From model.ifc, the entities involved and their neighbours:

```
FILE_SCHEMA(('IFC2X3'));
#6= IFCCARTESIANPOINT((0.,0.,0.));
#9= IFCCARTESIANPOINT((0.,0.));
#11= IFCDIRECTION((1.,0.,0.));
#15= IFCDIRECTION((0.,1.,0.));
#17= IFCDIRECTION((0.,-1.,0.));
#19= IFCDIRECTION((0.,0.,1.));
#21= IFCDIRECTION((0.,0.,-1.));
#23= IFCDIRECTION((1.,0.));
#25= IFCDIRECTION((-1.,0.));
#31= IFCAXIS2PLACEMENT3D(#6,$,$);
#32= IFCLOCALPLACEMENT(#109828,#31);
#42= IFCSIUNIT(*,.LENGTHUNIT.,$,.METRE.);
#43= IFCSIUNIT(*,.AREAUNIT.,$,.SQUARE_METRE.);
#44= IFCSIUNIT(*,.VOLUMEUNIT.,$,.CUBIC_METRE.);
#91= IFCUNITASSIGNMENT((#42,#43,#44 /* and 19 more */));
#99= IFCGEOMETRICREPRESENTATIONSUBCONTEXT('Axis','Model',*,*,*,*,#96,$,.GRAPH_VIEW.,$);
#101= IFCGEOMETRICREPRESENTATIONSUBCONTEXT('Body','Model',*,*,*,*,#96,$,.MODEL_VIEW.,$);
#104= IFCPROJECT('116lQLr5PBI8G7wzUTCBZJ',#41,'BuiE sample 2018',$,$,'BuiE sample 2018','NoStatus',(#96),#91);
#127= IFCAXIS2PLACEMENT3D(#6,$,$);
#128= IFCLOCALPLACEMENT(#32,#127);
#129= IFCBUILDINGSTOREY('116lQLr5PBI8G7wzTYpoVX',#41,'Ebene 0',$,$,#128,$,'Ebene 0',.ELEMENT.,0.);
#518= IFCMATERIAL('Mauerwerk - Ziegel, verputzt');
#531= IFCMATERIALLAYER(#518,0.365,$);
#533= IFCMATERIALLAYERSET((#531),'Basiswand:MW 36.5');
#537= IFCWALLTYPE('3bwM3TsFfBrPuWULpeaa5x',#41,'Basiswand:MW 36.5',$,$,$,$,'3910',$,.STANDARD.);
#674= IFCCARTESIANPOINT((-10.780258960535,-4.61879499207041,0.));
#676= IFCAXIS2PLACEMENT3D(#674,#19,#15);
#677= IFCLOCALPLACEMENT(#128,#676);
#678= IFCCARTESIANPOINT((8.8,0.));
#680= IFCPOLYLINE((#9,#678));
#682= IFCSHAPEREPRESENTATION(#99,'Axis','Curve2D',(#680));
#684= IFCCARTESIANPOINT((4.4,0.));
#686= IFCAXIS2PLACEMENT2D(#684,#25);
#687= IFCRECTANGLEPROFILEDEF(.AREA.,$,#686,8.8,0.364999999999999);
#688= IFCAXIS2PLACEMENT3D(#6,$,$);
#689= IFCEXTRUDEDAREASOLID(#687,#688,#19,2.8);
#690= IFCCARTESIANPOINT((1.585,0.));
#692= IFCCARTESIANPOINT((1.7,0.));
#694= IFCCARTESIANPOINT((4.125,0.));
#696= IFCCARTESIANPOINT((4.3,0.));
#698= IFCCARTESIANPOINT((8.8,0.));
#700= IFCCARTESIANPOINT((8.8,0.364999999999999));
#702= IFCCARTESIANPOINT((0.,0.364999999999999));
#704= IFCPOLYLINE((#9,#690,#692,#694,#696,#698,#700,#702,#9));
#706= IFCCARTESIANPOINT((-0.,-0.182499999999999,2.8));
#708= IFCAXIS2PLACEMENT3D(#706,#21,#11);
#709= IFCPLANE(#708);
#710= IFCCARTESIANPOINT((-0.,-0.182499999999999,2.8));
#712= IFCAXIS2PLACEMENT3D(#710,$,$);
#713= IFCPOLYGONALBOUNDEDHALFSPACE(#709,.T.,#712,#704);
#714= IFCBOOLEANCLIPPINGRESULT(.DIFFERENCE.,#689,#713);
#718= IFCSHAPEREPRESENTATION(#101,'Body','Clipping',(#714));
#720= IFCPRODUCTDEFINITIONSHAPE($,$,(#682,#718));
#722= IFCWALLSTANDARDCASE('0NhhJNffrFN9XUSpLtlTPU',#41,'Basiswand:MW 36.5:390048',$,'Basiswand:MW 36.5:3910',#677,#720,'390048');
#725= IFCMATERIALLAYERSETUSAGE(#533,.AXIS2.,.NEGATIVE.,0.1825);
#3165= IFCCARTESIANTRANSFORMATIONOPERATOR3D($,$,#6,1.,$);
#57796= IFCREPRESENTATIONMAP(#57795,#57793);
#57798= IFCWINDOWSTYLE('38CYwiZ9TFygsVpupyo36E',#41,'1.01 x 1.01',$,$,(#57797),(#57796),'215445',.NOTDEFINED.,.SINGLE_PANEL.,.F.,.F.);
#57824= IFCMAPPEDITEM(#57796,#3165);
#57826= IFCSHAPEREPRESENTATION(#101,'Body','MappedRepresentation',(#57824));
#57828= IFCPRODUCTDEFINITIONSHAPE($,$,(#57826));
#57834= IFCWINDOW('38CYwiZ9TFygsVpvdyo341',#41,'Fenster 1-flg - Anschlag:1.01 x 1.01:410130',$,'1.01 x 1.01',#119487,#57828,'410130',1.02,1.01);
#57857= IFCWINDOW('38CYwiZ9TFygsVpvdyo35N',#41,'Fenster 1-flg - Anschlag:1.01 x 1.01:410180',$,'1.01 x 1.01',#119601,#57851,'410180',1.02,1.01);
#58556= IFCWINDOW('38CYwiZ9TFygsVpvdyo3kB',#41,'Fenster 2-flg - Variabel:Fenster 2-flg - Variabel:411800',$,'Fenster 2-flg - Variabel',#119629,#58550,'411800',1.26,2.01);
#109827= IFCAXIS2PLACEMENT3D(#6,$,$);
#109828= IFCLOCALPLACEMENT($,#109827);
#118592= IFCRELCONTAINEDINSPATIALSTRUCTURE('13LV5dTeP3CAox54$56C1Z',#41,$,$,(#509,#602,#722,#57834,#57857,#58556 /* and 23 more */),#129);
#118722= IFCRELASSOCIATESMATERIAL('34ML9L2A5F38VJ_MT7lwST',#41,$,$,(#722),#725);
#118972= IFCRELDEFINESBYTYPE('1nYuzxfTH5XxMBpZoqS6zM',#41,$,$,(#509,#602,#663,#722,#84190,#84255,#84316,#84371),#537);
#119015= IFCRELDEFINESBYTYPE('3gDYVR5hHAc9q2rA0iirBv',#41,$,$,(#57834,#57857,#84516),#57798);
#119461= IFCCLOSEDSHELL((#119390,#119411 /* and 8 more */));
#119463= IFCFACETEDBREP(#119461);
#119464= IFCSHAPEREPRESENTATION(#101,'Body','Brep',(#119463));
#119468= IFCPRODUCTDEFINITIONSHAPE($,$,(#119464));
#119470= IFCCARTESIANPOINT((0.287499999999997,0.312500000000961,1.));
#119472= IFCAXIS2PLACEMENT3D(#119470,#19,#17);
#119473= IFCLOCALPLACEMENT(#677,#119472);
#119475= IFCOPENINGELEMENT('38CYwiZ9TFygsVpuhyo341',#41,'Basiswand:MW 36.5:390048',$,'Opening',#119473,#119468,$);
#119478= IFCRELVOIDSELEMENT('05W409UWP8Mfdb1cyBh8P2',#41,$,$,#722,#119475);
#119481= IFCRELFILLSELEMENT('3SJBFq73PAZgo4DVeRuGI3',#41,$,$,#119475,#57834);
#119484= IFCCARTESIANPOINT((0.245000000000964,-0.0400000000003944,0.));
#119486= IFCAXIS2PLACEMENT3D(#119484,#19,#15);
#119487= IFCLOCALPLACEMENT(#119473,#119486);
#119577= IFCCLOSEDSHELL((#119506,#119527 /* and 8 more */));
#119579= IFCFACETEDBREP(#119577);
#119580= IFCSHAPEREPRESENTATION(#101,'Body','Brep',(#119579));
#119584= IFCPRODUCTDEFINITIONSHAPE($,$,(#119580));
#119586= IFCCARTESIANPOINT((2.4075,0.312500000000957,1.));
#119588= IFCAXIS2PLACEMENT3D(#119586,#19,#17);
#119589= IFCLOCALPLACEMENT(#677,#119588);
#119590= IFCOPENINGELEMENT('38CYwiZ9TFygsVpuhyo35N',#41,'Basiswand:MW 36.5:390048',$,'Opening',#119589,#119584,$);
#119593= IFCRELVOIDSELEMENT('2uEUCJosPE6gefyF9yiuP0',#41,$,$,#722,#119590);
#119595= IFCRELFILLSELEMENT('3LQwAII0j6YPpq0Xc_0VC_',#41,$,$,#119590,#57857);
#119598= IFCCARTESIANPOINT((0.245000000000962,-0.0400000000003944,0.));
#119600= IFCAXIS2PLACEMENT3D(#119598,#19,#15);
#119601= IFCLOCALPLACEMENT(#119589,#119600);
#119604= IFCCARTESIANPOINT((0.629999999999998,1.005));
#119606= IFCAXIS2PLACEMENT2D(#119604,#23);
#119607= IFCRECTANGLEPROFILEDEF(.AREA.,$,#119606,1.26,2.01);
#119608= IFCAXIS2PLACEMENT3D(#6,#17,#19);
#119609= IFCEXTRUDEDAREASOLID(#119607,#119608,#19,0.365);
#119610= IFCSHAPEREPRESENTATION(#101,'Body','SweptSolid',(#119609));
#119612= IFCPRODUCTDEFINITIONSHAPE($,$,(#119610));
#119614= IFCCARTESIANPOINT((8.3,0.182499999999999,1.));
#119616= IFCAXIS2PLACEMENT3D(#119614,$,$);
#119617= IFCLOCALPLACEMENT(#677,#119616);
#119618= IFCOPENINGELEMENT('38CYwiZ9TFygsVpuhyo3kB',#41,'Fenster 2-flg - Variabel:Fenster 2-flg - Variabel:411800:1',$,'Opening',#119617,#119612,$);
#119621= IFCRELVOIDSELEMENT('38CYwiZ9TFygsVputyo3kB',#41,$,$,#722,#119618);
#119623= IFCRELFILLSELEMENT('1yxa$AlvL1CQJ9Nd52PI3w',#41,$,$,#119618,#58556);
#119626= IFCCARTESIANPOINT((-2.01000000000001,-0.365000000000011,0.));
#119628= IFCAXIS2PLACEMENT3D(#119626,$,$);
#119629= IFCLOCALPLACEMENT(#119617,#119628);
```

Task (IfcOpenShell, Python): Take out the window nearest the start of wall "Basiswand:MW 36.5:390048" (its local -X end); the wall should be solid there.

```python
import ifcopenshell
import ifcopenshell.api.feature
import ifcopenshell.api.root
import ifcopenshell.geom
import ifcopenshell.util.shape

model = ifcopenshell.open("model.ifc")
settings = ifcopenshell.geom.settings()


def volume(element):
    """Net volume in cubic metres, openings subtracted."""
    shape = ifcopenshell.geom.create_shape(settings, element)
    return ifcopenshell.util.shape.get_volume(shape.geometry)


window = model.by_id(57834)
opening = window.FillsVoids[0].RelatingOpeningElement
wall = opening.VoidsElements[0].RelatingBuildingElement
before = volume(wall)

ifcopenshell.api.root.remove_product(model, product=window)
ifcopenshell.api.feature.remove_feature(model, feature=opening)

after = volume(wall)

print(f"wall volume {before:.3f} -> {after:.3f} m3")

model.write("model-out.ifc")
```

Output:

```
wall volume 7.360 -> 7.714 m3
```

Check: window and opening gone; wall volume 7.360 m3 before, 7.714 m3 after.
